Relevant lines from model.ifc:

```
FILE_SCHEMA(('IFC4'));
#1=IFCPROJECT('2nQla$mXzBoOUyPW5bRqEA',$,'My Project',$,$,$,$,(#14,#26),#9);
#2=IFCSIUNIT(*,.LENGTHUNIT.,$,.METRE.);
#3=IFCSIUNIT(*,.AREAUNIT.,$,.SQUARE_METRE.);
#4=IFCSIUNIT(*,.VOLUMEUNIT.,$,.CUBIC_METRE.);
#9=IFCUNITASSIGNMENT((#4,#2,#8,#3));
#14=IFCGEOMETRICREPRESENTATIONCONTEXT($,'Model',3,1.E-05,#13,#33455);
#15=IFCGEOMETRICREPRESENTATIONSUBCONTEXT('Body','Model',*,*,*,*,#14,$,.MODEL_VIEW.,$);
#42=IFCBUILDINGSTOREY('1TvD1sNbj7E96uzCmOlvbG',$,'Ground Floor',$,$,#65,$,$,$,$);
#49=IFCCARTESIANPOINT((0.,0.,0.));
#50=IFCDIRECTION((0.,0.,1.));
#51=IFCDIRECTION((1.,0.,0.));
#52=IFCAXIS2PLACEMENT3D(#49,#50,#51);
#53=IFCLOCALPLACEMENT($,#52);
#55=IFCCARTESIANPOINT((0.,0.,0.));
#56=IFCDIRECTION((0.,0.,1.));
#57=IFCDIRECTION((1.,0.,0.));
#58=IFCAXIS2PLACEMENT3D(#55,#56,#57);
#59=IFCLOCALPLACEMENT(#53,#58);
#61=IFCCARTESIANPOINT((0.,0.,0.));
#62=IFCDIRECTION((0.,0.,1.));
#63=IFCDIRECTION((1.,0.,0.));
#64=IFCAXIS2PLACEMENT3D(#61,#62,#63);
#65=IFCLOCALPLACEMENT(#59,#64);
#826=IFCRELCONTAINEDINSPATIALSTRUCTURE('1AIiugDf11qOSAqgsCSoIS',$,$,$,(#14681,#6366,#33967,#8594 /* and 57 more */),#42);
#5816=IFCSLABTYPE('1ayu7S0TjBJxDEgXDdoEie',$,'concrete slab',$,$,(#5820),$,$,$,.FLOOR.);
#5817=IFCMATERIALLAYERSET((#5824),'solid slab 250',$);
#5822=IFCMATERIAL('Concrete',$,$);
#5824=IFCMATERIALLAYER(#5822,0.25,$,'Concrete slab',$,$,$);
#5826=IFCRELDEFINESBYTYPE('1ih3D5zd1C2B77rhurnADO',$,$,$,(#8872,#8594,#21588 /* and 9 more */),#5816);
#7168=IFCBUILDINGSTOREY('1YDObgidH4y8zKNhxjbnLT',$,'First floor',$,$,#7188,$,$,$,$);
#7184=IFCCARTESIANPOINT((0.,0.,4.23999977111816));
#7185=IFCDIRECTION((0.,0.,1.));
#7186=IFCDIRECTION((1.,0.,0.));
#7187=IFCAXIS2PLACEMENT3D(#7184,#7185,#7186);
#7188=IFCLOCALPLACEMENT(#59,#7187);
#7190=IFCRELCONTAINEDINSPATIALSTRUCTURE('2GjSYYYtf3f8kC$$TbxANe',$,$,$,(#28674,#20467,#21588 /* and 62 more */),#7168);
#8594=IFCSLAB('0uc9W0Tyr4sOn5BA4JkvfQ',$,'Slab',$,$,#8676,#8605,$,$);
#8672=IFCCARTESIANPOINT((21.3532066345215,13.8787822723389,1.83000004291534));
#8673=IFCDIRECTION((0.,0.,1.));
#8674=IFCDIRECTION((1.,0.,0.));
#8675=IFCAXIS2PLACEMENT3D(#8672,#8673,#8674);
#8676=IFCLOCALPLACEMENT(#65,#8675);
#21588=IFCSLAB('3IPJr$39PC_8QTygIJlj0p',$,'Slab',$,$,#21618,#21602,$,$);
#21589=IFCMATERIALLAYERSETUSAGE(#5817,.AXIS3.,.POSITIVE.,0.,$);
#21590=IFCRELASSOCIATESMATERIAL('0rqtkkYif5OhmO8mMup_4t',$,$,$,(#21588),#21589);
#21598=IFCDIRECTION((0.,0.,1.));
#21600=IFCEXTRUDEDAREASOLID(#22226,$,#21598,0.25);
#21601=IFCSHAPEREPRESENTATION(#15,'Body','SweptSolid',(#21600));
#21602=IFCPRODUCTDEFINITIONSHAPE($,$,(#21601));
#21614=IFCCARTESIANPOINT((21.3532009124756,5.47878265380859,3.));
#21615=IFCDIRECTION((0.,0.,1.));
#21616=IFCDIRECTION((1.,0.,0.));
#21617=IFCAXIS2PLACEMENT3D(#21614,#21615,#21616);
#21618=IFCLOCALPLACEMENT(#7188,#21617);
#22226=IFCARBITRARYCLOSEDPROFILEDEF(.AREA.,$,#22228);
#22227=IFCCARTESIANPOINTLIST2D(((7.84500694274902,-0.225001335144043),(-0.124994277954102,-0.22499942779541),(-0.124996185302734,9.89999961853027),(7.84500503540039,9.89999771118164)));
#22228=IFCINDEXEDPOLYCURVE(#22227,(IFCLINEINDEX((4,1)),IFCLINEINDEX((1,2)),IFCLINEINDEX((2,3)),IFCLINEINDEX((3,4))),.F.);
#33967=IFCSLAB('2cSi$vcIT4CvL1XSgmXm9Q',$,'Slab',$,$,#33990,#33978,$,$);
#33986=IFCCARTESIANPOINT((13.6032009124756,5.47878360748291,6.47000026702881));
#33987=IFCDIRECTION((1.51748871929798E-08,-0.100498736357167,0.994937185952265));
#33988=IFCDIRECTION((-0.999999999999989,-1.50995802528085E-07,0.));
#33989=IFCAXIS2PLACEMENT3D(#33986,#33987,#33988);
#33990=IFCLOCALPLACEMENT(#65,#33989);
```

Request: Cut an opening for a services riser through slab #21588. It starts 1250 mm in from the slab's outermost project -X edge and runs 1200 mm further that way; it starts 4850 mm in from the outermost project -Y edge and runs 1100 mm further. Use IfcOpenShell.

```python
import numpy as np
import ifcopenshell
import ifcopenshell.api.feature
import ifcopenshell.api.geometry
import ifcopenshell.api.root
import ifcopenshell.geom
import ifcopenshell.util.placement
import ifcopenshell.util.representation
import ifcopenshell.util.shape
import ifcopenshell.util.unit

model = ifcopenshell.open("model.ifc")
unit_scale = ifcopenshell.util.unit.calculate_unit_scale(model)
settings = ifcopenshell.geom.settings()


def volume(element):
    """Net volume in cubic metres, openings subtracted."""
    shape = ifcopenshell.geom.create_shape(settings, element)
    return ifcopenshell.util.shape.get_volume(shape.geometry)


slab = model.by_id(21588)
before = volume(slab)

# Extent in the slab's own axes, in metres. The edges named are its -X and -Y sides.
slab_shape = ifcopenshell.geom.create_shape(settings, slab)
vertices = ifcopenshell.util.shape.get_vertices(slab_shape.geometry)
x_min, y_min, bottom = vertices.min(axis=0)
top = vertices[:, 2].max()

opening = ifcopenshell.api.root.create_entity(model, ifc_class="IfcOpeningElement", name="Services riser opening", predefined_type="OPENING")
context = ifcopenshell.util.representation.get_context(model, "Model", "Body", "MODEL_VIEW")
width, depth = 1.2, 1.1
outline = [(0.0, 0.0), (width, 0.0), (width, depth), (0.0, depth), (0.0, 0.0)]
# Overshoot both faces by 50 mm so the cut is clean.
shape = ifcopenshell.api.geometry.add_slab_representation(
    model, context=context, depth=top - bottom + 0.1, polyline=outline
)
ifcopenshell.api.geometry.assign_representation(model, product=opening, representation=shape)

matrix = ifcopenshell.util.placement.get_local_placement(slab.ObjectPlacement)
matrix[:, 3] = matrix @ np.append(np.array([x_min + 1.25, y_min + 4.85, bottom - 0.05]) / unit_scale, 1.0)
ifcopenshell.api.geometry.edit_object_placement(model, product=opening, matrix=matrix, is_si=False)
ifcopenshell.api.feature.add_feature(model, feature=opening, element=slab)

after = volume(slab)

print(f"slab volume {before:.3f} -> {after:.3f} m3")

model.write("model_updated.ifc")
```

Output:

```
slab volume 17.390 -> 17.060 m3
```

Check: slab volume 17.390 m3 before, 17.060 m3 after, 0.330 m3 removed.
